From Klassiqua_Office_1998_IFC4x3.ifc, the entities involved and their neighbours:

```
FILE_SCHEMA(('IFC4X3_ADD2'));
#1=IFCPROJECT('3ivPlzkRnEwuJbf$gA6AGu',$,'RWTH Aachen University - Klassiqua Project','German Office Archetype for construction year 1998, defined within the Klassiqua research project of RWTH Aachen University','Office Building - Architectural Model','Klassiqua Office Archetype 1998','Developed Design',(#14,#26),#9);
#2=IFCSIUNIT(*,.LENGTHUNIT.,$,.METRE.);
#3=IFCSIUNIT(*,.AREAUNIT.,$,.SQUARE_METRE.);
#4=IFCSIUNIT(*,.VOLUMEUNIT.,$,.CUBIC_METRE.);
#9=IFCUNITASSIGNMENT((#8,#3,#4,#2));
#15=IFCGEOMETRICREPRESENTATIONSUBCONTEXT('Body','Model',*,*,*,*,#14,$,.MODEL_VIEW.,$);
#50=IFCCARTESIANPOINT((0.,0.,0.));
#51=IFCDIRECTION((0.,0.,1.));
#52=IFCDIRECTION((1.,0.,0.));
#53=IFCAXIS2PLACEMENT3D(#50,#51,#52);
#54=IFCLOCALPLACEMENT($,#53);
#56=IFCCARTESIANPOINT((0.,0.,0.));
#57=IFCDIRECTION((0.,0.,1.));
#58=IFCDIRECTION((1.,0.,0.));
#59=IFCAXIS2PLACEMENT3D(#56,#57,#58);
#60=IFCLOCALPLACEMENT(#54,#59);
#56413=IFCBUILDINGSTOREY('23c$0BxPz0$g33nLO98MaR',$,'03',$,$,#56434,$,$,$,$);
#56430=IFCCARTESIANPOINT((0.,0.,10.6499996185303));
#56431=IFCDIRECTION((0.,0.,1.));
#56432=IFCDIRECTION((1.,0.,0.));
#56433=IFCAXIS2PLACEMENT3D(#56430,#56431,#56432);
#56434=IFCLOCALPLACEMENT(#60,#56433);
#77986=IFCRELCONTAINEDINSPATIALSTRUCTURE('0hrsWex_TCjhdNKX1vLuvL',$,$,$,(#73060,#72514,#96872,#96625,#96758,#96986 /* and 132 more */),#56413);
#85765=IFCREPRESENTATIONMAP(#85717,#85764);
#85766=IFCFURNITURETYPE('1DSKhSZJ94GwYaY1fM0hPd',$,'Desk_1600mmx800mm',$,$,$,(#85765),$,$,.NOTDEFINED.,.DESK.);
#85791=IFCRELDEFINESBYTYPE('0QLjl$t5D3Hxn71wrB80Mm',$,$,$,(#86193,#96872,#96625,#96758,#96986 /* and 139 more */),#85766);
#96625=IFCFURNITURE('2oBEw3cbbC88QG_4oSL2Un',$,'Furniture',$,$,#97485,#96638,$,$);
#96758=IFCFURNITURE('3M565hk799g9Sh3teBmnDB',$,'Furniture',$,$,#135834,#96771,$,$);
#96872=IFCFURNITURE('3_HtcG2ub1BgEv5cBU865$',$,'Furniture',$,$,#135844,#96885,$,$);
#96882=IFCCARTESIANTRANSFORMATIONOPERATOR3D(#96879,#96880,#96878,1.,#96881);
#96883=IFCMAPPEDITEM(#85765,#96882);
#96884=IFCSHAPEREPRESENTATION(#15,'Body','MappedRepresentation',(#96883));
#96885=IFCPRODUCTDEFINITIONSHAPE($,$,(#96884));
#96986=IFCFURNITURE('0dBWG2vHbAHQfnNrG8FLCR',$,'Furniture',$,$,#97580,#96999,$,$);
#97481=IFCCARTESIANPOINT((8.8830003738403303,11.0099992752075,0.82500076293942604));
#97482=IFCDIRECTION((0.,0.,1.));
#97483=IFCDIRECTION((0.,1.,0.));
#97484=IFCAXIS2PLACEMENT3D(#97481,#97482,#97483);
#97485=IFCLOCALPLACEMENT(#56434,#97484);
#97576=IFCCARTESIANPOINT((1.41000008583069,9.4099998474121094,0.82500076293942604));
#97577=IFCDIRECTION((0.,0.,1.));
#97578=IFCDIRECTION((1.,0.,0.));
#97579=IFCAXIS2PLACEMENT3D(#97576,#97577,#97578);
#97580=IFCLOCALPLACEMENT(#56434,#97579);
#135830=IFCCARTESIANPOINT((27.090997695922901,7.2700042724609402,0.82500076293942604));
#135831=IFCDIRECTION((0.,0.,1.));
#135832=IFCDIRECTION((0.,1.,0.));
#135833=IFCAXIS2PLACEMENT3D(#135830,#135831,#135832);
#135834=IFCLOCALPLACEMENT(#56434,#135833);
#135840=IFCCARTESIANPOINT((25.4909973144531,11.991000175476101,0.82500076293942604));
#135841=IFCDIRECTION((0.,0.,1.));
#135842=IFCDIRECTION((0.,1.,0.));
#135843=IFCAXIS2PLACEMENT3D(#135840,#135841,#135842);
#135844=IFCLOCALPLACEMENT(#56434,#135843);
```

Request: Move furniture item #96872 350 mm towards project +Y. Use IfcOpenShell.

```python
import ifcopenshell
import ifcopenshell.api.geometry
import ifcopenshell.util.placement

model = ifcopenshell.open("Klassiqua_Office_1998_IFC4x3.ifc")

item = model.by_guid("3_HtcG2ub1BgEv5cBU865$")
matrix = ifcopenshell.util.placement.get_local_placement(item.ObjectPlacement)
matrix[1, 3] += 0.35
ifcopenshell.api.geometry.edit_object_placement(model, product=item, matrix=matrix, is_si=False)

print(ifcopenshell.util.placement.get_local_placement(item.ObjectPlacement).round(3) + 0.0)

model.write("Klassiqua_Office_1998_IFC4x3_rev.ifc")
```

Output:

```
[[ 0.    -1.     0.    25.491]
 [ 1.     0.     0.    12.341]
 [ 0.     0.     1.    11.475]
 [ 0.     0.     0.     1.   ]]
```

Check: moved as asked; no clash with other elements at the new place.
